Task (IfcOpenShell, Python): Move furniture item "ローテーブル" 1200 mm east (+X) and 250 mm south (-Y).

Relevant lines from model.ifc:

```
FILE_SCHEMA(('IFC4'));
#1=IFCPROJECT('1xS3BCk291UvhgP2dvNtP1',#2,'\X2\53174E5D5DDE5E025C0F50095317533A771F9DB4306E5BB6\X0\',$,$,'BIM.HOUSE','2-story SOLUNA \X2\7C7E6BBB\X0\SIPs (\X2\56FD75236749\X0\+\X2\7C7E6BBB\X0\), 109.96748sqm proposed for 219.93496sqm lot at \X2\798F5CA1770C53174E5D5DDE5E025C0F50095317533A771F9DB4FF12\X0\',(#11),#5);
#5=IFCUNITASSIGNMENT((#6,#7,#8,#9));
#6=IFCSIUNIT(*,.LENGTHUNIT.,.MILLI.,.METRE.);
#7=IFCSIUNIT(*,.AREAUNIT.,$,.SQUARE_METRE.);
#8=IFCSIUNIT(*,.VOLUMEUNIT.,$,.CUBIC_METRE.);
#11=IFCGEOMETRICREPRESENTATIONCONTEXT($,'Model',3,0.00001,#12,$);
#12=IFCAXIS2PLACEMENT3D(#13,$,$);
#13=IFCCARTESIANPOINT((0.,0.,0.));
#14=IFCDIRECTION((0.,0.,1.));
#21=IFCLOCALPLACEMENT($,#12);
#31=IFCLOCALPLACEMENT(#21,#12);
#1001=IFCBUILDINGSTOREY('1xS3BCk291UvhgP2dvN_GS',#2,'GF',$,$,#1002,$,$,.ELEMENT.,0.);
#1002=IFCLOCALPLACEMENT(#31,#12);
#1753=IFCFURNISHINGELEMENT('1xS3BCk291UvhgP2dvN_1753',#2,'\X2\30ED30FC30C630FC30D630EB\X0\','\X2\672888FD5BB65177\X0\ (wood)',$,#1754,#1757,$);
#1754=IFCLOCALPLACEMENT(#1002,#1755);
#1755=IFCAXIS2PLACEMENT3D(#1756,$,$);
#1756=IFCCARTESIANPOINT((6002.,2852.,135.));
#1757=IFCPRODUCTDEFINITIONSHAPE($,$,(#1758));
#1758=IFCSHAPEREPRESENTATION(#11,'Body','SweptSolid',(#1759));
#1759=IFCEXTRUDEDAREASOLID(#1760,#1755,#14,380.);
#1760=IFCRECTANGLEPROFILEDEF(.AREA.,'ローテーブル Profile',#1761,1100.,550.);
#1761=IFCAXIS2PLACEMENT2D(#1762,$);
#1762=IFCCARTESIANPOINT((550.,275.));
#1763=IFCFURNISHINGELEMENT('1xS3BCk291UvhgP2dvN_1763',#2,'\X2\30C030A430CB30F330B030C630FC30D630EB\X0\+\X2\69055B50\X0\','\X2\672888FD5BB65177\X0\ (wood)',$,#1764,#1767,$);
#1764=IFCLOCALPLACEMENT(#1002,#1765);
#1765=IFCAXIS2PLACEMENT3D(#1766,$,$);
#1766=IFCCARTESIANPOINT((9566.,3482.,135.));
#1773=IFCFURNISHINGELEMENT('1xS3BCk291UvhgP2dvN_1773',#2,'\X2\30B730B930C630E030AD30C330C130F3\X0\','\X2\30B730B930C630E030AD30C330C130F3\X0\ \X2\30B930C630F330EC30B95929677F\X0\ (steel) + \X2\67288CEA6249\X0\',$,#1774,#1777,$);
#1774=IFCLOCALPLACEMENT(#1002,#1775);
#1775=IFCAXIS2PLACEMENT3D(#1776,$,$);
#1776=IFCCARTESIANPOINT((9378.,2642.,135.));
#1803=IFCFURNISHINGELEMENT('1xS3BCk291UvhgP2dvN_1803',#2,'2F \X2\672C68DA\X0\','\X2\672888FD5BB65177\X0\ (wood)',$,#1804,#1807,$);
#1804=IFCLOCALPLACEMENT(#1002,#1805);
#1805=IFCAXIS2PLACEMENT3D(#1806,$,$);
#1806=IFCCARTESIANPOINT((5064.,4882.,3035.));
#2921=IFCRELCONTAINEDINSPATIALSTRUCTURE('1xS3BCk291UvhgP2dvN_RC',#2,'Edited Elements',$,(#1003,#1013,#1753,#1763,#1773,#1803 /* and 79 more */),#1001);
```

```python
import ifcopenshell
import ifcopenshell.api.geometry
import ifcopenshell.util.placement
import ifcopenshell.util.unit

model = ifcopenshell.open("model.ifc")
unit_scale = ifcopenshell.util.unit.calculate_unit_scale(model)

item = model.by_id(1753)
matrix = ifcopenshell.util.placement.get_local_placement(item.ObjectPlacement)
matrix[0, 3] += 1.2 / unit_scale
matrix[1, 3] -= 0.25 / unit_scale
ifcopenshell.api.geometry.edit_object_placement(model, product=item, matrix=matrix, is_si=False)

print(ifcopenshell.util.placement.get_local_placement(item.ObjectPlacement).round(3) + 0.0)

model.write("model-out.ifc")
```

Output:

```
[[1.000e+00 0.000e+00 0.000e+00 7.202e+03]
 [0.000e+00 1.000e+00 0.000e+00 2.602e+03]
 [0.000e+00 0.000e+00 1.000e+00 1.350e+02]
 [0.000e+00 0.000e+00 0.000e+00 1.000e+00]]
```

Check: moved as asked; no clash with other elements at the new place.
